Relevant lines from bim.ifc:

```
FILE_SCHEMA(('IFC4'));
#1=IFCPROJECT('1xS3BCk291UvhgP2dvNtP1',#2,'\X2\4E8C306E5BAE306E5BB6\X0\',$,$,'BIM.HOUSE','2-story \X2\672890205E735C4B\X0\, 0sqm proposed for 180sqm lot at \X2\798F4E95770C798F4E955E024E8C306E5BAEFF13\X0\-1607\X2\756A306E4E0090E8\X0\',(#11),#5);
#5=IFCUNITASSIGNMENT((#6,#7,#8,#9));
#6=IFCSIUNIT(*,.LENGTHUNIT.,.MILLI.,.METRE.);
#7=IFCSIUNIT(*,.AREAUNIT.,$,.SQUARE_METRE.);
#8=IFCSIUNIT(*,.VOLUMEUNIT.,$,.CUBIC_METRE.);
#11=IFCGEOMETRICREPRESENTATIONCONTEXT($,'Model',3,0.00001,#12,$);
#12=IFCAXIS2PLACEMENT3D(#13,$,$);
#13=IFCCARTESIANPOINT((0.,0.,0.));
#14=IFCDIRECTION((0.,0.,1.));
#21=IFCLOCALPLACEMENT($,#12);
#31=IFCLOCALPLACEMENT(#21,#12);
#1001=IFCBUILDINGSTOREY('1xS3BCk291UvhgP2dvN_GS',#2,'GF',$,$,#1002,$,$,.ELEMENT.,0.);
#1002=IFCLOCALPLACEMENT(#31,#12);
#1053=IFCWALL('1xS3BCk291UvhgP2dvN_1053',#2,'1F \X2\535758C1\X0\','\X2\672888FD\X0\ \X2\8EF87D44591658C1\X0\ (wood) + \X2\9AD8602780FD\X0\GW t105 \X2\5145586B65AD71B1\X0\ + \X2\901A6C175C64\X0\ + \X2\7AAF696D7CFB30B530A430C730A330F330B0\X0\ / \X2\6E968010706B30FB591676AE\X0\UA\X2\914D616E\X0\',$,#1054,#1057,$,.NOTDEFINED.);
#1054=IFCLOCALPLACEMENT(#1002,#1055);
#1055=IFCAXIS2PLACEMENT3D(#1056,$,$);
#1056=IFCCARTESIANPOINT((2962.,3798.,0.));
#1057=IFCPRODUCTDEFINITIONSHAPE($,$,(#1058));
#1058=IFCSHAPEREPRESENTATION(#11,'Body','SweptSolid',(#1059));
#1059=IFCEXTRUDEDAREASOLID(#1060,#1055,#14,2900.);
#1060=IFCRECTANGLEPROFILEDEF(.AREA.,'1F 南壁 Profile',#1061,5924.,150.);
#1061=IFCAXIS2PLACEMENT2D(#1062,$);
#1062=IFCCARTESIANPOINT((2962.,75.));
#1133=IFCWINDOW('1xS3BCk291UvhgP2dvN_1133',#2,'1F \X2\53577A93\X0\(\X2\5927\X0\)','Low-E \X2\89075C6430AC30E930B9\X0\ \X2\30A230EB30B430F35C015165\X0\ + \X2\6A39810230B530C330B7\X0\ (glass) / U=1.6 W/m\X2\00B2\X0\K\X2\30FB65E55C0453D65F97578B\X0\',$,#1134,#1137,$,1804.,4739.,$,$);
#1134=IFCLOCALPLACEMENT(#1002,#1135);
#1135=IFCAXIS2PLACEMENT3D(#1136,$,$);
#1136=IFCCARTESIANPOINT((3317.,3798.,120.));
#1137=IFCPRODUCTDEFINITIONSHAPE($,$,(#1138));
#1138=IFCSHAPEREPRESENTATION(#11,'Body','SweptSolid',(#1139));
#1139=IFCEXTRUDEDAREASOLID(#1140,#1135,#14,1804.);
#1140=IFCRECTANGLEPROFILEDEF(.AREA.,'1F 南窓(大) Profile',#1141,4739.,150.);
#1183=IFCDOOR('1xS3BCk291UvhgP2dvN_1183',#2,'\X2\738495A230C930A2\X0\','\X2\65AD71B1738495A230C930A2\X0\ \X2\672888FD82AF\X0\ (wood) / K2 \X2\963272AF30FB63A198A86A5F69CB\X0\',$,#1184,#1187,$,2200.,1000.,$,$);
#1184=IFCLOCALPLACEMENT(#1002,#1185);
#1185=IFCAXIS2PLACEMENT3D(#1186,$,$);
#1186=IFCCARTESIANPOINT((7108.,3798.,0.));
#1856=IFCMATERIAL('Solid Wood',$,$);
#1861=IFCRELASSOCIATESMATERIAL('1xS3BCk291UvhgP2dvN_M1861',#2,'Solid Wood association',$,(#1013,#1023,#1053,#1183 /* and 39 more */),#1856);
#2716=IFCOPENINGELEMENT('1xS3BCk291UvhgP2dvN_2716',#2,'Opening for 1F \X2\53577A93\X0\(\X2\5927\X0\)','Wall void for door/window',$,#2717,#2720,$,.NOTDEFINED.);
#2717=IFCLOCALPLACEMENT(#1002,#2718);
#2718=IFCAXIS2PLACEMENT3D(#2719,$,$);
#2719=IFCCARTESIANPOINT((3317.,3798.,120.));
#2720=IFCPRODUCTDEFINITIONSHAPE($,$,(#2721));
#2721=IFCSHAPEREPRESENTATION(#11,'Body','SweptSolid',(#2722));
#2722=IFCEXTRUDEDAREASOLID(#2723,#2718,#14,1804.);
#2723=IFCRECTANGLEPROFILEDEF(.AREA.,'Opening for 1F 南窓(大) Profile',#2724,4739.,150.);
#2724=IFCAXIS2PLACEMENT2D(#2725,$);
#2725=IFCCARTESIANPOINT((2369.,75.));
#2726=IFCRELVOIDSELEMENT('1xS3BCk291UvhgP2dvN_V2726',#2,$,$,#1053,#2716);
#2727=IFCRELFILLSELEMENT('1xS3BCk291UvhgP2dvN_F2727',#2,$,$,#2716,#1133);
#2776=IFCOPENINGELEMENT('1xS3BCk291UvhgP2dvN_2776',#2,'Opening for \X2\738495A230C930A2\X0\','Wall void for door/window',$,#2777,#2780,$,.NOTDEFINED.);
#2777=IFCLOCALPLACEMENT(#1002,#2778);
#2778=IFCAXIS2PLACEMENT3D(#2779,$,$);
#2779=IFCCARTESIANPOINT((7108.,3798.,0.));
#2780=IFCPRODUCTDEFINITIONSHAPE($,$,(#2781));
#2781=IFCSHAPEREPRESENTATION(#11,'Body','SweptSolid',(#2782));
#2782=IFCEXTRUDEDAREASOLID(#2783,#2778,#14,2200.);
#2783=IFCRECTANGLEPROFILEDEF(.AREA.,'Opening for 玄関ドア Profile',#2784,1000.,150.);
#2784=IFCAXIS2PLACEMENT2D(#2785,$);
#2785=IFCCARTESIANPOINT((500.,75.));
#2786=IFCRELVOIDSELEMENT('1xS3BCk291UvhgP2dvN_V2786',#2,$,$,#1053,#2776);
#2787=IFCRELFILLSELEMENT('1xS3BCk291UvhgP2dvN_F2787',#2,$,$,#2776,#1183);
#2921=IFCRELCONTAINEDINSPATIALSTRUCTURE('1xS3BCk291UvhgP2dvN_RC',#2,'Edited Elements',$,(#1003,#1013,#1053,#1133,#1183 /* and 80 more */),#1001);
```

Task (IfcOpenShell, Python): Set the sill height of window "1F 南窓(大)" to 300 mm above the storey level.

```python
import numpy as np
import ifcopenshell
import ifcopenshell.api.geometry
import ifcopenshell.geom
import ifcopenshell.util.element
import ifcopenshell.util.placement
import ifcopenshell.util.shape
import ifcopenshell.util.unit

model = ifcopenshell.open("bim.ifc")
unit_scale = ifcopenshell.util.unit.calculate_unit_scale(model)

window = model.by_guid("1xS3BCk291UvhgP2dvN_1133")
opening = window.FillsVoids[0].RelatingOpeningElement
storey = ifcopenshell.util.element.get_container(window, ifc_class="IfcBuildingStorey")
level = ifcopenshell.util.placement.get_local_placement(storey.ObjectPlacement)[2, 3]

# The opening's origin need not be at the sill, so measure its lowest point.
shape = ifcopenshell.geom.create_shape(ifcopenshell.geom.settings(), opening)
bottom = ifcopenshell.util.shape.get_shape_bottom_elevation(shape, shape.geometry) / unit_scale
dz = level + 300.0 - bottom

shift = np.array([0.0, 0.0, dz])
# The window is not placed relative to its opening, so move both.
for product in (opening, window):
    matrix = ifcopenshell.util.placement.get_local_placement(product.ObjectPlacement)
    matrix[:3, 3] += shift
    ifcopenshell.api.geometry.edit_object_placement(model, product=product, matrix=matrix, is_si=False)

print(f"moved by {dz * unit_scale:+.3f} m")

model.write("bim_v2.ifc")
```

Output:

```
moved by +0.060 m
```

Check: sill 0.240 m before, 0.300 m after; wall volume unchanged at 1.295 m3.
